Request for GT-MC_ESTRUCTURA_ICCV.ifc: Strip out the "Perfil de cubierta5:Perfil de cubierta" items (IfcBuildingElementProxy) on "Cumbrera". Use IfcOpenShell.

First a look at what the model holds.

```python
import ifcopenshell
import ifcopenshell.util.element

model = ifcopenshell.open("GT-MC_ESTRUCTURA_ICCV.ifc")
print(model.schema)
storey = next(s for s in model.by_type("IfcBuildingStorey") if s.Name == "Cumbrera")
proxies = [e for e in ifcopenshell.util.element.get_decomposition(storey) if e.is_a("IfcBuildingElementProxy")]
seen = {}
for e in proxies:
    element_type = ifcopenshell.util.element.get_type(e)
    name = element_type.Name if element_type not in (None, e) else None
    seen[name] = seen.get(name, 0) + 1
for name, count in sorted(seen.items(), key=str):
    print(count, "x", name)
```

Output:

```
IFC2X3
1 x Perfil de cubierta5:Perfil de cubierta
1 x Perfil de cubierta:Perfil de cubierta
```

```python
import ifcopenshell
import ifcopenshell.api.root
import ifcopenshell.util.element

model = ifcopenshell.open("GT-MC_ESTRUCTURA_ICCV.ifc")

storey = next(s for s in model.by_type("IfcBuildingStorey") if s.Name == "Cumbrera")
proxies = [e for e in ifcopenshell.util.element.get_decomposition(storey) if e.is_a("IfcBuildingElementProxy")]
targets = [e for e in proxies if (t := ifcopenshell.util.element.get_type(e)) not in (None, e) and t.Name == "Perfil de cubierta5:Perfil de cubierta"]

for e in targets:
    ifcopenshell.api.root.remove_product(model, product=e)
print(len(targets), "removed")

model.write("GT-MC_ESTRUCTURA_ICCV-out.ifc")
```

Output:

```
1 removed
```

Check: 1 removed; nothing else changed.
